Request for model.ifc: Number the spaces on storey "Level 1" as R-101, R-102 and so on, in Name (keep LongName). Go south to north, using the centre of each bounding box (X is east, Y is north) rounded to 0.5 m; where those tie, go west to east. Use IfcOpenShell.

First a look at what the model holds.

```python
import ifcopenshell
import ifcopenshell.util.element
import ifcopenshell.util.placement

model = ifcopenshell.open("model.ifc")
print(model.schema)
storey = next(s for s in model.by_type("IfcBuildingStorey") if s.Name == "Level 1")
spaces = [e for e in ifcopenshell.util.element.get_decomposition(storey) if e.is_a("IfcSpace")]
for e in sorted(spaces, key=lambda e: e.id()):
    origin = ifcopenshell.util.placement.get_local_placement(e.ObjectPlacement)[:3, 3]
    print(e.id(), e.Name, e.LongName, origin.round(2) + 0.0, sep=" | ")
```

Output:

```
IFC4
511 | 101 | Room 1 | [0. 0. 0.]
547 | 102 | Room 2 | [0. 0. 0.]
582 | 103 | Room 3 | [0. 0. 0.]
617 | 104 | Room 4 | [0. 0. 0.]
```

```python
import ifcopenshell
import ifcopenshell.geom
import ifcopenshell.util.element
import ifcopenshell.util.shape

model = ifcopenshell.open("model.ifc")
settings = ifcopenshell.geom.settings()
settings.set("use-world-coords", True)


def centre(element):
    shape = ifcopenshell.geom.create_shape(settings, element)
    return ifcopenshell.util.shape.get_bbox_centroid(shape.geometry)


storey = next(s for s in model.by_type("IfcBuildingStorey") if s.Name == "Level 1")
spaces = [e for e in ifcopenshell.util.element.get_decomposition(storey) if e.is_a("IfcSpace")]

# Insertion points can sit at a corner or the storey origin, so sort by the geometry (in metres).
centres = {e: centre(e) for e in spaces}
spaces.sort(key=lambda e: (round(centres[e][1] / 0.5), centres[e][0]))

for i, e in enumerate(spaces, start=1):
    number = f"R-1{i:02d}"
    e.Name = number
    print(e.id(), number)

model.write("model_v2.ifc")
```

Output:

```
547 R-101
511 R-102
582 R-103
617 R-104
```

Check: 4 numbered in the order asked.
